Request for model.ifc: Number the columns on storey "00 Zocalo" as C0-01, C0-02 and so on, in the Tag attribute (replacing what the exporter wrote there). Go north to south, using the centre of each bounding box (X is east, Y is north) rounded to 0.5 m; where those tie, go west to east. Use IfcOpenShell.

First a look at what the model holds.

```python
import ifcopenshell
import ifcopenshell.util.element
import ifcopenshell.util.placement

model = ifcopenshell.open("model.ifc")
print(model.schema)
storey = next(s for s in model.by_type("IfcBuildingStorey") if s.Name == "00 Zocalo")
columns = [e for e in ifcopenshell.util.element.get_decomposition(storey) if e.is_a("IfcColumn")]
for e in sorted(columns, key=lambda e: e.id()):
    origin = ifcopenshell.util.placement.get_local_placement(e.ObjectPlacement)[:3, 3]
    print(e.id(), e.Tag, e.Name, origin.round(2) + 0.0, sep=" | ")
```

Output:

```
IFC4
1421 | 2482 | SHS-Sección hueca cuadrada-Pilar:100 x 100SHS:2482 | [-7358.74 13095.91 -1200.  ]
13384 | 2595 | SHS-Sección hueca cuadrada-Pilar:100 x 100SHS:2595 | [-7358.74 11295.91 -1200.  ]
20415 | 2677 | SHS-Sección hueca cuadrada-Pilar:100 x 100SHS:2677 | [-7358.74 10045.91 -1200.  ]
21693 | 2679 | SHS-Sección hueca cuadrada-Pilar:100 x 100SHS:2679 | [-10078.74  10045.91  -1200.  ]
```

```python
import ifcopenshell
import ifcopenshell.geom
import ifcopenshell.util.element
import ifcopenshell.util.shape

model = ifcopenshell.open("model.ifc")
settings = ifcopenshell.geom.settings()
settings.set("use-world-coords", True)


def centre(element):
    shape = ifcopenshell.geom.create_shape(settings, element)
    return ifcopenshell.util.shape.get_bbox_centroid(shape.geometry)


storey = next(s for s in model.by_type("IfcBuildingStorey") if s.Name == "00 Zocalo")
columns = [e for e in ifcopenshell.util.element.get_decomposition(storey) if e.is_a("IfcColumn")]

# Insertion points can sit at a corner or the storey origin, so sort by the geometry (in metres).
centres = {e: centre(e) for e in columns}
columns.sort(key=lambda e: (-round(centres[e][1] / 0.5), centres[e][0]))

for i, e in enumerate(columns, start=1):
    number = f"C0-{i:02d}"
    e.Tag = number
    print(e.id(), number)

model.write("model_rev.ifc")
```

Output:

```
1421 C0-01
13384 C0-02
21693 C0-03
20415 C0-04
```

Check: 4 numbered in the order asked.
